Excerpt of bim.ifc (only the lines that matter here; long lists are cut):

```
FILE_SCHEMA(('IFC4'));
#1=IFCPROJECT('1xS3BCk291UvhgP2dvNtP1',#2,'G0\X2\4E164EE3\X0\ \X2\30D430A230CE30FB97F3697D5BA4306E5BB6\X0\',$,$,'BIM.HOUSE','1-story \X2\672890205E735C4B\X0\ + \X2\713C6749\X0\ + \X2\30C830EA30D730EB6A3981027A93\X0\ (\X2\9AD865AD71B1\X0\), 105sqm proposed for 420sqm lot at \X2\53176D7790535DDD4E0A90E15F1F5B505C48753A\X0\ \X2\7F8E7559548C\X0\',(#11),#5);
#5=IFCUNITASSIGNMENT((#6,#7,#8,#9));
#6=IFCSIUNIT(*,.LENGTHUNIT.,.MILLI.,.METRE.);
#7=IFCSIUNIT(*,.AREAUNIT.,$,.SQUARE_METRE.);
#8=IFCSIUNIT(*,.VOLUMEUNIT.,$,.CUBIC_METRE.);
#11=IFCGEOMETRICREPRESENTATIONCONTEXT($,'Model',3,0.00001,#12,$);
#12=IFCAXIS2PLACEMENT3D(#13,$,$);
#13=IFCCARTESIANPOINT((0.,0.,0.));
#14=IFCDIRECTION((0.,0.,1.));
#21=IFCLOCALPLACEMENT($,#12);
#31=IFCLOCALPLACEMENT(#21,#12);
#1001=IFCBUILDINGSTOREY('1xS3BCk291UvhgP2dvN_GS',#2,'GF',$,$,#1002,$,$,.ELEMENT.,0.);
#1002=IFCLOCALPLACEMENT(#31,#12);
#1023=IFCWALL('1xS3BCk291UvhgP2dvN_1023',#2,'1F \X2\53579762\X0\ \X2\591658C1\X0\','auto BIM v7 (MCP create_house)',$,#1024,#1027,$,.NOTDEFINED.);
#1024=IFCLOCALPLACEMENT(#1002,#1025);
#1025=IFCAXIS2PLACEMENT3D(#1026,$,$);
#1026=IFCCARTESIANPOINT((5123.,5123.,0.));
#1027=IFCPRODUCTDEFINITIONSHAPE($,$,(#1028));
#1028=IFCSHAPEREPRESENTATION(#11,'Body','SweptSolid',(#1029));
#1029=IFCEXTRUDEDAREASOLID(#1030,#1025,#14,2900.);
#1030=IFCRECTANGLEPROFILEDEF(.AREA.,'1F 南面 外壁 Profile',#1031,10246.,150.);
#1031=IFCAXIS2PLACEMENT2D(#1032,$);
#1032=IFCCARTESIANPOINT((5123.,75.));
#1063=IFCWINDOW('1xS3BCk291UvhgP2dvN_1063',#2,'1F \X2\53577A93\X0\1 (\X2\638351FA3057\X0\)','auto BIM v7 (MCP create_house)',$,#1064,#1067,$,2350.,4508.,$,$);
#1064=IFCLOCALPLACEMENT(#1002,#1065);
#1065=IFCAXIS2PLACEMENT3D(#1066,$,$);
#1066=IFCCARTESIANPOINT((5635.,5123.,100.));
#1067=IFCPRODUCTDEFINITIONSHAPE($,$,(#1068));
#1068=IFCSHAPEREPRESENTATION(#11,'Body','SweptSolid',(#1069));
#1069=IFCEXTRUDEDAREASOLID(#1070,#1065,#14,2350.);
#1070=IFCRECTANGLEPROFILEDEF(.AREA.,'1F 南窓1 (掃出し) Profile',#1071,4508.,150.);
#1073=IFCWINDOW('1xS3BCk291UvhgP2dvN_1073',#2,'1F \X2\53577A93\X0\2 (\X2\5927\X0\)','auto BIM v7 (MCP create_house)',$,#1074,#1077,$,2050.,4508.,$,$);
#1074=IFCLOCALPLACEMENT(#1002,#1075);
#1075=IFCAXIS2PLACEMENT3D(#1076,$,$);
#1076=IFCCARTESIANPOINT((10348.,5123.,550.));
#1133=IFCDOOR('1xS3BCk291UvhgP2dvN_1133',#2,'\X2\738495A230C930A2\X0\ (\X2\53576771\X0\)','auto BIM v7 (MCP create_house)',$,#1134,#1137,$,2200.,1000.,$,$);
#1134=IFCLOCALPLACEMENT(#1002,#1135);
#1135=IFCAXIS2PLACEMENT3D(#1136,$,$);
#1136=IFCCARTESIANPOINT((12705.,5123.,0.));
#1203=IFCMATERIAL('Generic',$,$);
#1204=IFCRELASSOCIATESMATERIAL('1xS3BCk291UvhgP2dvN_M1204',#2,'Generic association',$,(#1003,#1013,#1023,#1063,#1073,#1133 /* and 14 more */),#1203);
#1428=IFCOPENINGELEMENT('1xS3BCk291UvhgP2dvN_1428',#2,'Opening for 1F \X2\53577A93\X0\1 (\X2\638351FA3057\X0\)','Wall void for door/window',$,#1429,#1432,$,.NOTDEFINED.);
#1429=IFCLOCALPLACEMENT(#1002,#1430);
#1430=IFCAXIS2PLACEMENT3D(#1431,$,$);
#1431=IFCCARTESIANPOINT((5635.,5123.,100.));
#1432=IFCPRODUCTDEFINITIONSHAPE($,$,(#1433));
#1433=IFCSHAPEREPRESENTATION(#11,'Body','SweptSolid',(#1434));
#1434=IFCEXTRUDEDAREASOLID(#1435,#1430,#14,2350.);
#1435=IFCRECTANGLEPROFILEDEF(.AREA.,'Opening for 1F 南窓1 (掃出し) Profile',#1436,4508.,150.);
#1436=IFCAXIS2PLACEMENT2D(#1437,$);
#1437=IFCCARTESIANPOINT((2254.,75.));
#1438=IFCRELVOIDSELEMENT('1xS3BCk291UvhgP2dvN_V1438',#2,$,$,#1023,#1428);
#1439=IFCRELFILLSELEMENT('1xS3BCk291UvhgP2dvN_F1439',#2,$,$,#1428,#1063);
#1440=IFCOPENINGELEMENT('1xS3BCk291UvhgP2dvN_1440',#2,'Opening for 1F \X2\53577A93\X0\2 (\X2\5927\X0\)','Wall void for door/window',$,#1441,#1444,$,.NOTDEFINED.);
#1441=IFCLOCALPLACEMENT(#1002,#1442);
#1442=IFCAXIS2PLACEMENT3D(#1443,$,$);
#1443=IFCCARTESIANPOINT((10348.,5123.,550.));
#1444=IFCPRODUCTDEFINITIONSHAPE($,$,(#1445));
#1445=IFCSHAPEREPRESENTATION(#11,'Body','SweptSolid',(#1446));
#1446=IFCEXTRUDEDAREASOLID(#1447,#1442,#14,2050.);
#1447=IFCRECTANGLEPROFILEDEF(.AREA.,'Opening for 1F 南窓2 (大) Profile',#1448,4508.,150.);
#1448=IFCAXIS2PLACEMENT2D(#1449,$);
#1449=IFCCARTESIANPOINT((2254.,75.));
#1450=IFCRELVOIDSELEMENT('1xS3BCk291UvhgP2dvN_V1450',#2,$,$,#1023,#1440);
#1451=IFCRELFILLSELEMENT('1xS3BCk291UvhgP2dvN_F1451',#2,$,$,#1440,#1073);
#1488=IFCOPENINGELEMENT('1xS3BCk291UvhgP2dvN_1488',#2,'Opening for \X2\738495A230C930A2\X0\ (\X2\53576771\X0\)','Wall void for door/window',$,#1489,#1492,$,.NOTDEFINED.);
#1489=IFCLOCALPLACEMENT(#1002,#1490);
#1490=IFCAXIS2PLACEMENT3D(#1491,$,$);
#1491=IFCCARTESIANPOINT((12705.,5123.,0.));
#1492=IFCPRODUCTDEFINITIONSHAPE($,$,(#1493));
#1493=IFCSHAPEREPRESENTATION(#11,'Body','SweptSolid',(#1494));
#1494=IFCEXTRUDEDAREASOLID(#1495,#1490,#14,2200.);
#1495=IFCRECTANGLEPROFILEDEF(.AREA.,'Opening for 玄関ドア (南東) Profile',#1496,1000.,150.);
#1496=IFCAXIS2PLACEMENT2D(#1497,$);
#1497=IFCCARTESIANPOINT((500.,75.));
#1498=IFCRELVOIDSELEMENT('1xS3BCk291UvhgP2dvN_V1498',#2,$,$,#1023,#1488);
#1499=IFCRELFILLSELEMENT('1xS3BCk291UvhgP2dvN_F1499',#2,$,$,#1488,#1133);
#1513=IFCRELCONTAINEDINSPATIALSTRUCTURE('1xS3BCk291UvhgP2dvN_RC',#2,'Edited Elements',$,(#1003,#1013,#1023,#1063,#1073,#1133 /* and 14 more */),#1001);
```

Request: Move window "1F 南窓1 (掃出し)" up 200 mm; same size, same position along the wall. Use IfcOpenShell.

```python
import numpy as np
import ifcopenshell
import ifcopenshell.api.geometry
import ifcopenshell.util.placement
import ifcopenshell.util.unit

model = ifcopenshell.open("bim.ifc")
unit_scale = ifcopenshell.util.unit.calculate_unit_scale(model)

window = model.by_guid("1xS3BCk291UvhgP2dvN_1063")
opening = window.FillsVoids[0].RelatingOpeningElement
dz = 0.2 / unit_scale

shift = np.array([0.0, 0.0, dz])
# The window is not placed relative to its opening, so move both.
for product in (opening, window):
    matrix = ifcopenshell.util.placement.get_local_placement(product.ObjectPlacement)
    matrix[:3, 3] += shift
    ifcopenshell.api.geometry.edit_object_placement(model, product=product, matrix=matrix, is_si=False)

print(f"moved by {dz * unit_scale:+.3f} m")

model.write("bim_v2.ifc")
```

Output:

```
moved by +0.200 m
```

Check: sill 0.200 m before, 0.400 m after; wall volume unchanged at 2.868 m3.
